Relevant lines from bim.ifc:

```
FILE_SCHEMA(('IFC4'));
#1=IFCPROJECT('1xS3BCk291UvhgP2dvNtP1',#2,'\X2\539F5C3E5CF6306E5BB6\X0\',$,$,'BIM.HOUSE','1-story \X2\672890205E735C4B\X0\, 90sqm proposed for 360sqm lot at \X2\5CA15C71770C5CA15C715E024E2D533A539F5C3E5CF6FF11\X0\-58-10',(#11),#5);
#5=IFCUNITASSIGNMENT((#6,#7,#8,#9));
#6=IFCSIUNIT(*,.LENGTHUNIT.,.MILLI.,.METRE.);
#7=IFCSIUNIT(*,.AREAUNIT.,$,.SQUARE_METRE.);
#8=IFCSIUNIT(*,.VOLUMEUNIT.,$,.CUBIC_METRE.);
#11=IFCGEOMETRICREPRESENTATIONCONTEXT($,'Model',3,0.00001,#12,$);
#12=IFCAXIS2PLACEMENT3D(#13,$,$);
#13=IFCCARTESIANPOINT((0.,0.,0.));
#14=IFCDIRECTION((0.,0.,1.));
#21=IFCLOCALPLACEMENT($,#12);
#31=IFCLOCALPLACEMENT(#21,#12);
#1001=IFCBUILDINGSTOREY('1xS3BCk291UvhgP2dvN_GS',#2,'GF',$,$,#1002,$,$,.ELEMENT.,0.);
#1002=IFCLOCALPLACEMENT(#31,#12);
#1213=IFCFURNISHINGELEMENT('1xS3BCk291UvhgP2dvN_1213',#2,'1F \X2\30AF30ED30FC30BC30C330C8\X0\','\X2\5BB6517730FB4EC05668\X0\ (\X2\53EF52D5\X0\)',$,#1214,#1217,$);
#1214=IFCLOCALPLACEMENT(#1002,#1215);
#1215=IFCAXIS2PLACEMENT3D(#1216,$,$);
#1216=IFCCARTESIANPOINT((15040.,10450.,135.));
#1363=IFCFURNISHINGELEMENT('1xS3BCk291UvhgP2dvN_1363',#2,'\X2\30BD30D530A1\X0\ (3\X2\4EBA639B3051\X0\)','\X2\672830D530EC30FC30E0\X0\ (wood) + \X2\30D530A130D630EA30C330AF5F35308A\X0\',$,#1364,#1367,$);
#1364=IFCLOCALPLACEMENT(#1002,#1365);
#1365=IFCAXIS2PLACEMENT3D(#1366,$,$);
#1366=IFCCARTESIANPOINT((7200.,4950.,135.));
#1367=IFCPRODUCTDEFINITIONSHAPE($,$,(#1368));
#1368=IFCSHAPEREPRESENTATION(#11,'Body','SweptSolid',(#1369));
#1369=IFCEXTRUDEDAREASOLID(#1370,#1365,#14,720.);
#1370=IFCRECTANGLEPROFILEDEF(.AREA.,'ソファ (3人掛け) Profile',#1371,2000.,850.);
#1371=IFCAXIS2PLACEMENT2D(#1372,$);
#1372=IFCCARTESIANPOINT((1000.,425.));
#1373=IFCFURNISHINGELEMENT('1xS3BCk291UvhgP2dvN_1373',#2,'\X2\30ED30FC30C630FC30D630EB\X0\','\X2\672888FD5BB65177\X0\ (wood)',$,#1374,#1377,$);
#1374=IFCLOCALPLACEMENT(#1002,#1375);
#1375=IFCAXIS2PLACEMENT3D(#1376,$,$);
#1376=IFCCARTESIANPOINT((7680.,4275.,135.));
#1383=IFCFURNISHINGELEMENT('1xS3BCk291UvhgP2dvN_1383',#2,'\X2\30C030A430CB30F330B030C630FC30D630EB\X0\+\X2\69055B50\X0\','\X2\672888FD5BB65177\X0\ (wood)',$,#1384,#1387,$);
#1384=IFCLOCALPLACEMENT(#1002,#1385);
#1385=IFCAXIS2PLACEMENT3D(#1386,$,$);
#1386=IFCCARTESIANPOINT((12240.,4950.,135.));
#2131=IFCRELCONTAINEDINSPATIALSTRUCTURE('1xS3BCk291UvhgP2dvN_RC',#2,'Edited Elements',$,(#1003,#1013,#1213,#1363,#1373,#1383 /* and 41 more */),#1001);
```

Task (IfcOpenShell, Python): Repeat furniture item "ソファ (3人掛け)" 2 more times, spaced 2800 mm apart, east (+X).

```python
import numpy as np
import ifcopenshell
import ifcopenshell.api.geometry
import ifcopenshell.api.root
import ifcopenshell.util.element
import ifcopenshell.util.placement

model = ifcopenshell.open("bim.ifc")


def reuse_history(source, copy):
    """copy_class also copies each property set's owner history, people and application; keep the originals."""
    for rel in copy.IsDefinedBy:
        if rel.is_a("IfcRelDefinesByProperties") and (history := rel.RelatingPropertyDefinition.OwnerHistory):
            rel.RelatingPropertyDefinition.OwnerHistory = source.OwnerHistory
            ifcopenshell.util.element.remove_deep2(model, history)


source = model.by_guid("1xS3BCk291UvhgP2dvN_1363")
base = ifcopenshell.util.placement.get_local_placement(source.ObjectPlacement)
step = np.array([1.0, 0.0, 0.0]) * 2800.0

for i in range(1, 3):
    copy = ifcopenshell.api.root.copy_class(model, product=source)
    copy.Representation = ifcopenshell.util.element.copy_deep(
        model, source.Representation, exclude=["IfcGeometricRepresentationContext", "IfcRepresentationMap"]
    )
    reuse_history(source, copy)
    matrix = base.copy()
    matrix[:3, 3] += i * step
    print("added at", matrix[:3, 3].round(3) + 0.0)
    ifcopenshell.api.geometry.edit_object_placement(model, product=copy, matrix=matrix, is_si=False)

model.write("bim_v2.ifc")
```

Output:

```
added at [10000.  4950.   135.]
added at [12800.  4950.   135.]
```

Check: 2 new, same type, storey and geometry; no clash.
